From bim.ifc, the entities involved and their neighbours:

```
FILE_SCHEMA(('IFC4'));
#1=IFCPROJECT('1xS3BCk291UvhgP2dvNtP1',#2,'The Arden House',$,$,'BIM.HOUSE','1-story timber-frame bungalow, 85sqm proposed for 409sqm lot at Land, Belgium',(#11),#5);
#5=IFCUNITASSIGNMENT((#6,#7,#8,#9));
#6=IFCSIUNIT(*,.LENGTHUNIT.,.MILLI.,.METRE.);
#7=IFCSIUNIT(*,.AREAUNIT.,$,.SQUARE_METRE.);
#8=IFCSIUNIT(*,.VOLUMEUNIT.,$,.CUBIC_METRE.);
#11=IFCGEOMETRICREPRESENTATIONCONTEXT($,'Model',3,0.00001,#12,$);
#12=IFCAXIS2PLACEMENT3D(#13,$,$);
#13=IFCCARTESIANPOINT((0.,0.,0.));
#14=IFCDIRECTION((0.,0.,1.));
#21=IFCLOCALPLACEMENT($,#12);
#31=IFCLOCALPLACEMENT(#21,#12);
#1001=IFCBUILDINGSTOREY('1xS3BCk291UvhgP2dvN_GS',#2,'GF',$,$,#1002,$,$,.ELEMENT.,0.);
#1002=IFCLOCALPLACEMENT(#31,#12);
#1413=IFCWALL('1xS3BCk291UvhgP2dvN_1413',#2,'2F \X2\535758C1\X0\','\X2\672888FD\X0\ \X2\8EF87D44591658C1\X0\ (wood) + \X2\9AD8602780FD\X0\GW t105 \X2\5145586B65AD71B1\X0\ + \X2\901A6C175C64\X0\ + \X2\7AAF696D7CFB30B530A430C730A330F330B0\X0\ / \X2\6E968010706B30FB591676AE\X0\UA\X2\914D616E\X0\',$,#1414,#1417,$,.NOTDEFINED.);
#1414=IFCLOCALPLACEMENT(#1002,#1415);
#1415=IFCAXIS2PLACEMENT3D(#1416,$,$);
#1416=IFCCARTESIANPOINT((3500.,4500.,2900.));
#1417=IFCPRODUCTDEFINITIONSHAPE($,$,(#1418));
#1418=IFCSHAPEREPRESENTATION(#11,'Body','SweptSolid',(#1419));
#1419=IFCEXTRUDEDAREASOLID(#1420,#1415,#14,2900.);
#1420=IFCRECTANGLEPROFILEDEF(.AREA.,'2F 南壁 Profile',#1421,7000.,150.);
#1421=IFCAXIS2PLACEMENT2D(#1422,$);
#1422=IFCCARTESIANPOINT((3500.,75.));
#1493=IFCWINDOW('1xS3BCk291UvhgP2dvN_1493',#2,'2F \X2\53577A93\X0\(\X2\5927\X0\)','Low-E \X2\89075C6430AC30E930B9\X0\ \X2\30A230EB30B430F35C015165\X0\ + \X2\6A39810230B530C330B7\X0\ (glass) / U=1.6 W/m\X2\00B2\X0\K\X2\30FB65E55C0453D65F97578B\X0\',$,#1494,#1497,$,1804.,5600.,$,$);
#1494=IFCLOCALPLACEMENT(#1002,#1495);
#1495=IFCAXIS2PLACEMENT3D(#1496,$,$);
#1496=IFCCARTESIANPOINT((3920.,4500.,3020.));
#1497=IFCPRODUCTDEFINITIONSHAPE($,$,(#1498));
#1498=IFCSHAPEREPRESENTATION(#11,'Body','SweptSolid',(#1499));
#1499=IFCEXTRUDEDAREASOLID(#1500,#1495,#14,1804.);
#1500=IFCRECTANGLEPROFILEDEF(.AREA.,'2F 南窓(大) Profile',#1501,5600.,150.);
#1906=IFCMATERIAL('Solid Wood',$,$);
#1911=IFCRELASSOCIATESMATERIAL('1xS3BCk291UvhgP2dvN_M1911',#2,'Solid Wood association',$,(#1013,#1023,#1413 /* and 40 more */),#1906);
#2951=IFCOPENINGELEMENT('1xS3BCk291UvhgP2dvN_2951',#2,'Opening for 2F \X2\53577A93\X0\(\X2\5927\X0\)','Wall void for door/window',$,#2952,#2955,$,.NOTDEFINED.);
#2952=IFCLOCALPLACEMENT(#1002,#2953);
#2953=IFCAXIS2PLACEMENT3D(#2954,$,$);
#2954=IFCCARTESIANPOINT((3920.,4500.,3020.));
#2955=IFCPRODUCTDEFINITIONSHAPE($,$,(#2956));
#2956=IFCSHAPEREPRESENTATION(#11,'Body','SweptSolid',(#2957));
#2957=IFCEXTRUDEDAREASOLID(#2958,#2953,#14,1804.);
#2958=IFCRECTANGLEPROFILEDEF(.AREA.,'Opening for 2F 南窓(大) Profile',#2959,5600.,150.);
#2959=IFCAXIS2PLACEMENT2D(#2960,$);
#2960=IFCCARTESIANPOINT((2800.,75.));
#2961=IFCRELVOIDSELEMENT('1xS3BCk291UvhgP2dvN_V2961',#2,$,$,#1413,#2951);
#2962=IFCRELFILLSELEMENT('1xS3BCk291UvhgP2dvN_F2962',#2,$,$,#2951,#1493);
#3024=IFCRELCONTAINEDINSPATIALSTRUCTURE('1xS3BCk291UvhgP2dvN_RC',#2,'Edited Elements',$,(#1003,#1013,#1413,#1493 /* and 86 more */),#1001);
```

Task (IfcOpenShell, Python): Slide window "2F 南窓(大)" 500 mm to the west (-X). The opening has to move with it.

```python
import ifcopenshell
import ifcopenshell.api.geometry
import ifcopenshell.util.placement

model = ifcopenshell.open("bim.ifc")

window = model.by_id(1493)
opening = window.FillsVoids[0].RelatingOpeningElement
wall = opening.VoidsElements[0].RelatingBuildingElement

wall_matrix = ifcopenshell.util.placement.get_local_placement(wall.ObjectPlacement)
shift = wall_matrix[:3, 0] * -500.0
before = ifcopenshell.util.placement.get_local_placement(window.ObjectPlacement)[:3, 3].copy()

# The window is not placed relative to its opening, so move both.
for product in (opening, window):
    matrix = ifcopenshell.util.placement.get_local_placement(product.ObjectPlacement)
    matrix[:3, 3] += shift
    ifcopenshell.api.geometry.edit_object_placement(model, product=product, matrix=matrix, is_si=False)

after = ifcopenshell.util.placement.get_local_placement(window.ObjectPlacement)[:3, 3]
print("window moved by", (after - before).round(3) + 0.0)

model.write("bim-out.ifc")
```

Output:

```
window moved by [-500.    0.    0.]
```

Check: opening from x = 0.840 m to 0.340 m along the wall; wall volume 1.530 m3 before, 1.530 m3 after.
